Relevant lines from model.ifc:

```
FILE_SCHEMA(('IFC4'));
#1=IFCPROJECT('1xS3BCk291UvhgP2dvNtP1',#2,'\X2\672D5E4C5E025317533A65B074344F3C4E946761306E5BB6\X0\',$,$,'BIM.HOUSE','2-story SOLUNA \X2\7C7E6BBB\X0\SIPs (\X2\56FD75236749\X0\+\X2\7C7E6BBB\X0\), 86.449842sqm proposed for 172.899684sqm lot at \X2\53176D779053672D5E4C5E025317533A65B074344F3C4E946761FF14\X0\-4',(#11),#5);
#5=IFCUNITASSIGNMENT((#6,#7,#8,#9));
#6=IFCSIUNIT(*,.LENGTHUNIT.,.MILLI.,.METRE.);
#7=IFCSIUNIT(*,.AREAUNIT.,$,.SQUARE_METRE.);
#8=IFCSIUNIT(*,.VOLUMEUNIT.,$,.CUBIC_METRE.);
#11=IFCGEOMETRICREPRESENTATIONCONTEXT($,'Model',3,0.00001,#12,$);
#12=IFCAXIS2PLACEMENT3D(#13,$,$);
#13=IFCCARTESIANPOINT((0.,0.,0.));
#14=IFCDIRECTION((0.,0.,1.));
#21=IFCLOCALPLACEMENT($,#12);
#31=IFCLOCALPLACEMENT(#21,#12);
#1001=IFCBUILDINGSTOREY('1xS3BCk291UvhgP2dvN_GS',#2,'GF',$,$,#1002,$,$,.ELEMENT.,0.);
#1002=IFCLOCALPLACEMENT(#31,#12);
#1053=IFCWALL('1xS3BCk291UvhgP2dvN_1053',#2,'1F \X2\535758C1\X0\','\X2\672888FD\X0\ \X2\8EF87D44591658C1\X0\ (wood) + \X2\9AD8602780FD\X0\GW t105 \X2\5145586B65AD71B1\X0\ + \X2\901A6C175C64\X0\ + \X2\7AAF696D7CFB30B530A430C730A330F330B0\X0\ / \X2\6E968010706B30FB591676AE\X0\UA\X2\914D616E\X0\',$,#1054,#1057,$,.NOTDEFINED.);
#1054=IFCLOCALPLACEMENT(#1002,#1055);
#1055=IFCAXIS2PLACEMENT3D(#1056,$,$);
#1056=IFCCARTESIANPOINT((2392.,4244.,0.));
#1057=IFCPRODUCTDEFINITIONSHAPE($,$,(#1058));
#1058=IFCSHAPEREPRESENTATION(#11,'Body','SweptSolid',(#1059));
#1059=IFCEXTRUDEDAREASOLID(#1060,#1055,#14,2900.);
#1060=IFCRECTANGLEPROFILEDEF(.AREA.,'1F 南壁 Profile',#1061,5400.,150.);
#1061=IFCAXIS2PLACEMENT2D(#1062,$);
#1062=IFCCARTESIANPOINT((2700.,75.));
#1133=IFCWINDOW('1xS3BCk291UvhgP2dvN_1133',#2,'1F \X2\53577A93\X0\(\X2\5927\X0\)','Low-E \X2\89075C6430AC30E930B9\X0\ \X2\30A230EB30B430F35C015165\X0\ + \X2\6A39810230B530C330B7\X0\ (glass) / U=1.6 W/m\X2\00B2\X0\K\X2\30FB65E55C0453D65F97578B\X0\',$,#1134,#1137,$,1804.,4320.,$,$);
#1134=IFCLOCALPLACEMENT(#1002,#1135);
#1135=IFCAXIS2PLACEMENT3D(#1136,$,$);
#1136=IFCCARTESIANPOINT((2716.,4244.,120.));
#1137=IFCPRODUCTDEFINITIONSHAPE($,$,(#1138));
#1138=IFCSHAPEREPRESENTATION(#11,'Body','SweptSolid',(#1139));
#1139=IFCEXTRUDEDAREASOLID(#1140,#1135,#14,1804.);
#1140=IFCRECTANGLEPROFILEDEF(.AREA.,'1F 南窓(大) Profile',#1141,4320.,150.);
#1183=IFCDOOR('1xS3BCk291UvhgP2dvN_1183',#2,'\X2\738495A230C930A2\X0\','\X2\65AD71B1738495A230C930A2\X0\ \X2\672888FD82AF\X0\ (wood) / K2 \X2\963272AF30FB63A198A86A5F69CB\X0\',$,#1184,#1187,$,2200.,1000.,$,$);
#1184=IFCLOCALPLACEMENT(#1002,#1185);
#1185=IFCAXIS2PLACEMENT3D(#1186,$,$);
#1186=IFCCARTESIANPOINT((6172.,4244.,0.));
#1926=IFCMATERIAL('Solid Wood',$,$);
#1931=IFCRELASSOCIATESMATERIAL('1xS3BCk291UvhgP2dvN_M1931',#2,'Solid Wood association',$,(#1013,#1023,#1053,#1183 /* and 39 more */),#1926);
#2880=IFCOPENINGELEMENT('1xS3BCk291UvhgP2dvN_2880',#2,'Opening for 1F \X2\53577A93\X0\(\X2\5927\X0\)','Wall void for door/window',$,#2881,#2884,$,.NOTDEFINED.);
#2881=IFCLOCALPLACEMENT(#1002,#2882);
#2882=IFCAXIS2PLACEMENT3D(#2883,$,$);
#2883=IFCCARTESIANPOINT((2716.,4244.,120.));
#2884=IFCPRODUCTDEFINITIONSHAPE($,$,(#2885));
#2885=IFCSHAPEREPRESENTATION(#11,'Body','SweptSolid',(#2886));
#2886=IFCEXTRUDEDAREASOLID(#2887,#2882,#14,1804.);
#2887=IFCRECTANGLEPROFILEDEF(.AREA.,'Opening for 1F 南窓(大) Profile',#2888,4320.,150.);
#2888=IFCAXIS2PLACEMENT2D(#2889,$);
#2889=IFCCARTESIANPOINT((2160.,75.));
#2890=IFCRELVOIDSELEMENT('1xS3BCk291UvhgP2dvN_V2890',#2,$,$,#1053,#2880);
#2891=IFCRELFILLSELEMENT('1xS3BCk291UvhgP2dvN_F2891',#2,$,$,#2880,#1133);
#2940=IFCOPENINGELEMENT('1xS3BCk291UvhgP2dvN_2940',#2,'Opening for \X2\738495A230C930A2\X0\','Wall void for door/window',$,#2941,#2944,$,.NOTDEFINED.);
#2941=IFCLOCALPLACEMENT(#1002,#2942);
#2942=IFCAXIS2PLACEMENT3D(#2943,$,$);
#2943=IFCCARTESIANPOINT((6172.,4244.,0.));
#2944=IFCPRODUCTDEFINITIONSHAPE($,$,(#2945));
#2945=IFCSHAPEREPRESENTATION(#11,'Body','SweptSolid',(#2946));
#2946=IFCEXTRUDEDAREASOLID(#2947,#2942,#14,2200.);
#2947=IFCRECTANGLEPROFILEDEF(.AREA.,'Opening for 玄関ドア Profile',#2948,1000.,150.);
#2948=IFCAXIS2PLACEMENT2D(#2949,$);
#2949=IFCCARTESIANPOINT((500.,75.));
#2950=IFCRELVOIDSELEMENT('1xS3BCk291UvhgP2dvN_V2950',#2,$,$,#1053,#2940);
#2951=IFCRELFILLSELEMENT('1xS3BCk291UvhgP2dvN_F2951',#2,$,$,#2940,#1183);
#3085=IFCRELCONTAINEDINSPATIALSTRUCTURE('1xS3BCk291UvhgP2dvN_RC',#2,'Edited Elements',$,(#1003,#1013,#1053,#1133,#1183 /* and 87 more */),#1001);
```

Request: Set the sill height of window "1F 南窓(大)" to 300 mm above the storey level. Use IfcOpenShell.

```python
import numpy as np
import ifcopenshell
import ifcopenshell.api.geometry
import ifcopenshell.geom
import ifcopenshell.util.element
import ifcopenshell.util.placement
import ifcopenshell.util.shape
import ifcopenshell.util.unit

model = ifcopenshell.open("model.ifc")
unit_scale = ifcopenshell.util.unit.calculate_unit_scale(model)

window = model.by_guid("1xS3BCk291UvhgP2dvN_1133")
opening = window.FillsVoids[0].RelatingOpeningElement
storey = ifcopenshell.util.element.get_container(window, ifc_class="IfcBuildingStorey")
level = ifcopenshell.util.placement.get_local_placement(storey.ObjectPlacement)[2, 3]

# The opening's origin need not be at the sill, so measure its lowest point.
shape = ifcopenshell.geom.create_shape(ifcopenshell.geom.settings(), opening)
bottom = ifcopenshell.util.shape.get_shape_bottom_elevation(shape, shape.geometry) / unit_scale
dz = level + 300.0 - bottom

shift = np.array([0.0, 0.0, dz])
# The window is not placed relative to its opening, so move both.
for product in (opening, window):
    matrix = ifcopenshell.util.placement.get_local_placement(product.ObjectPlacement)
    matrix[:3, 3] += shift
    ifcopenshell.api.geometry.edit_object_placement(model, product=product, matrix=matrix, is_si=False)

print(f"moved by {dz * unit_scale:+.3f} m")

model.write("model_edited.ifc")
```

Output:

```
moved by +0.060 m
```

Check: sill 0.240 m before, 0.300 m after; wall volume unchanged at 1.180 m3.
